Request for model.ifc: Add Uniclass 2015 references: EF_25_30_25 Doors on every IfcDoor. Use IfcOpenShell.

First a look at what the model holds.

```python
import ifcopenshell

model = ifcopenshell.open("model.ifc")
print(model.schema)
print("classifications:", [c.Name for c in model.by_type("IfcClassification")])
for ifc_class in ("IfcDoor", "IfcRoof", "IfcStair", "IfcWall", "IfcWindow"):
    print(ifc_class, len(model.by_type(ifc_class)))
```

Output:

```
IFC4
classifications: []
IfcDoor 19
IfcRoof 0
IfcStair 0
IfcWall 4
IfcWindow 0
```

```python
import ifcopenshell
import ifcopenshell.api.classification

model = ifcopenshell.open("model.ifc")

system = ifcopenshell.api.classification.add_classification(model, classification="Uniclass 2015")

codes = {
    "IfcDoor": ("EF_25_30_25", "Doors"),
}
for ifc_class, (code, name) in codes.items():
    products = model.by_type(ifc_class)
    ifcopenshell.api.classification.add_reference(
        model, products=products, classification=system, identification=code, name=name
    )
    print(code, len(products))

model.write("model_rev.ifc")
```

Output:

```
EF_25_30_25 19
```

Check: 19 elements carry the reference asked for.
